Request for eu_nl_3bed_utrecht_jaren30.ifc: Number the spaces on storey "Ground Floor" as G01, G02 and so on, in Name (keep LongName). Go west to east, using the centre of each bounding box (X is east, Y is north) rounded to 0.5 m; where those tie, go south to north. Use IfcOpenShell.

First a look at what the model holds.

```python
import ifcopenshell
import ifcopenshell.util.element
import ifcopenshell.util.placement

model = ifcopenshell.open("eu_nl_3bed_utrecht_jaren30.ifc")
print(model.schema)
storey = next(s for s in model.by_type("IfcBuildingStorey") if s.Name == "Ground Floor")
spaces = [e for e in ifcopenshell.util.element.get_decomposition(storey) if e.is_a("IfcSpace")]
for e in sorted(spaces, key=lambda e: e.id()):
    origin = ifcopenshell.util.placement.get_local_placement(e.ObjectPlacement)[:3, 3]
    print(e.id(), e.Name, e.LongName, origin.round(2) + 0.0, sep=" | ")
```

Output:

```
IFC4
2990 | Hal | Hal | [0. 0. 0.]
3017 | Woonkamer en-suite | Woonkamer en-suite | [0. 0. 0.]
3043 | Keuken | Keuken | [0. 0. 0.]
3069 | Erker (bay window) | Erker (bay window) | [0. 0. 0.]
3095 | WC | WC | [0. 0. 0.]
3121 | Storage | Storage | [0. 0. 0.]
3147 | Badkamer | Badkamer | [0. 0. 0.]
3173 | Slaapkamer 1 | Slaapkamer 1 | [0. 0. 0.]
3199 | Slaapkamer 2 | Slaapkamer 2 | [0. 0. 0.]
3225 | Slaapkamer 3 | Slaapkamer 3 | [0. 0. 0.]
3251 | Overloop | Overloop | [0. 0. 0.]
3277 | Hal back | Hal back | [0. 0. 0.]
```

```python
import ifcopenshell
import ifcopenshell.geom
import ifcopenshell.util.element
import ifcopenshell.util.shape

model = ifcopenshell.open("eu_nl_3bed_utrecht_jaren30.ifc")
settings = ifcopenshell.geom.settings()
settings.set("use-world-coords", True)


def centre(element):
    shape = ifcopenshell.geom.create_shape(settings, element)
    return ifcopenshell.util.shape.get_bbox_centroid(shape.geometry)


storey = next(s for s in model.by_type("IfcBuildingStorey") if s.Name == "Ground Floor")
spaces = [e for e in ifcopenshell.util.element.get_decomposition(storey) if e.is_a("IfcSpace")]

# Insertion points can sit at a corner or the storey origin, so sort by the geometry (in metres).
centres = {e: centre(e) for e in spaces}
spaces.sort(key=lambda e: (round(centres[e][0] / 0.5), centres[e][1]))

for i, e in enumerate(spaces, start=1):
    number = f"G{i:02d}"
    e.Name = number
    print(e.id(), number)

model.write("eu_nl_3bed_utrecht_jaren30-out.ifc")
```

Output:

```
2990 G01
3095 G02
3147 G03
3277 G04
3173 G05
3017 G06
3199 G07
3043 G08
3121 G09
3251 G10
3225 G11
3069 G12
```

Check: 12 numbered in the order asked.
